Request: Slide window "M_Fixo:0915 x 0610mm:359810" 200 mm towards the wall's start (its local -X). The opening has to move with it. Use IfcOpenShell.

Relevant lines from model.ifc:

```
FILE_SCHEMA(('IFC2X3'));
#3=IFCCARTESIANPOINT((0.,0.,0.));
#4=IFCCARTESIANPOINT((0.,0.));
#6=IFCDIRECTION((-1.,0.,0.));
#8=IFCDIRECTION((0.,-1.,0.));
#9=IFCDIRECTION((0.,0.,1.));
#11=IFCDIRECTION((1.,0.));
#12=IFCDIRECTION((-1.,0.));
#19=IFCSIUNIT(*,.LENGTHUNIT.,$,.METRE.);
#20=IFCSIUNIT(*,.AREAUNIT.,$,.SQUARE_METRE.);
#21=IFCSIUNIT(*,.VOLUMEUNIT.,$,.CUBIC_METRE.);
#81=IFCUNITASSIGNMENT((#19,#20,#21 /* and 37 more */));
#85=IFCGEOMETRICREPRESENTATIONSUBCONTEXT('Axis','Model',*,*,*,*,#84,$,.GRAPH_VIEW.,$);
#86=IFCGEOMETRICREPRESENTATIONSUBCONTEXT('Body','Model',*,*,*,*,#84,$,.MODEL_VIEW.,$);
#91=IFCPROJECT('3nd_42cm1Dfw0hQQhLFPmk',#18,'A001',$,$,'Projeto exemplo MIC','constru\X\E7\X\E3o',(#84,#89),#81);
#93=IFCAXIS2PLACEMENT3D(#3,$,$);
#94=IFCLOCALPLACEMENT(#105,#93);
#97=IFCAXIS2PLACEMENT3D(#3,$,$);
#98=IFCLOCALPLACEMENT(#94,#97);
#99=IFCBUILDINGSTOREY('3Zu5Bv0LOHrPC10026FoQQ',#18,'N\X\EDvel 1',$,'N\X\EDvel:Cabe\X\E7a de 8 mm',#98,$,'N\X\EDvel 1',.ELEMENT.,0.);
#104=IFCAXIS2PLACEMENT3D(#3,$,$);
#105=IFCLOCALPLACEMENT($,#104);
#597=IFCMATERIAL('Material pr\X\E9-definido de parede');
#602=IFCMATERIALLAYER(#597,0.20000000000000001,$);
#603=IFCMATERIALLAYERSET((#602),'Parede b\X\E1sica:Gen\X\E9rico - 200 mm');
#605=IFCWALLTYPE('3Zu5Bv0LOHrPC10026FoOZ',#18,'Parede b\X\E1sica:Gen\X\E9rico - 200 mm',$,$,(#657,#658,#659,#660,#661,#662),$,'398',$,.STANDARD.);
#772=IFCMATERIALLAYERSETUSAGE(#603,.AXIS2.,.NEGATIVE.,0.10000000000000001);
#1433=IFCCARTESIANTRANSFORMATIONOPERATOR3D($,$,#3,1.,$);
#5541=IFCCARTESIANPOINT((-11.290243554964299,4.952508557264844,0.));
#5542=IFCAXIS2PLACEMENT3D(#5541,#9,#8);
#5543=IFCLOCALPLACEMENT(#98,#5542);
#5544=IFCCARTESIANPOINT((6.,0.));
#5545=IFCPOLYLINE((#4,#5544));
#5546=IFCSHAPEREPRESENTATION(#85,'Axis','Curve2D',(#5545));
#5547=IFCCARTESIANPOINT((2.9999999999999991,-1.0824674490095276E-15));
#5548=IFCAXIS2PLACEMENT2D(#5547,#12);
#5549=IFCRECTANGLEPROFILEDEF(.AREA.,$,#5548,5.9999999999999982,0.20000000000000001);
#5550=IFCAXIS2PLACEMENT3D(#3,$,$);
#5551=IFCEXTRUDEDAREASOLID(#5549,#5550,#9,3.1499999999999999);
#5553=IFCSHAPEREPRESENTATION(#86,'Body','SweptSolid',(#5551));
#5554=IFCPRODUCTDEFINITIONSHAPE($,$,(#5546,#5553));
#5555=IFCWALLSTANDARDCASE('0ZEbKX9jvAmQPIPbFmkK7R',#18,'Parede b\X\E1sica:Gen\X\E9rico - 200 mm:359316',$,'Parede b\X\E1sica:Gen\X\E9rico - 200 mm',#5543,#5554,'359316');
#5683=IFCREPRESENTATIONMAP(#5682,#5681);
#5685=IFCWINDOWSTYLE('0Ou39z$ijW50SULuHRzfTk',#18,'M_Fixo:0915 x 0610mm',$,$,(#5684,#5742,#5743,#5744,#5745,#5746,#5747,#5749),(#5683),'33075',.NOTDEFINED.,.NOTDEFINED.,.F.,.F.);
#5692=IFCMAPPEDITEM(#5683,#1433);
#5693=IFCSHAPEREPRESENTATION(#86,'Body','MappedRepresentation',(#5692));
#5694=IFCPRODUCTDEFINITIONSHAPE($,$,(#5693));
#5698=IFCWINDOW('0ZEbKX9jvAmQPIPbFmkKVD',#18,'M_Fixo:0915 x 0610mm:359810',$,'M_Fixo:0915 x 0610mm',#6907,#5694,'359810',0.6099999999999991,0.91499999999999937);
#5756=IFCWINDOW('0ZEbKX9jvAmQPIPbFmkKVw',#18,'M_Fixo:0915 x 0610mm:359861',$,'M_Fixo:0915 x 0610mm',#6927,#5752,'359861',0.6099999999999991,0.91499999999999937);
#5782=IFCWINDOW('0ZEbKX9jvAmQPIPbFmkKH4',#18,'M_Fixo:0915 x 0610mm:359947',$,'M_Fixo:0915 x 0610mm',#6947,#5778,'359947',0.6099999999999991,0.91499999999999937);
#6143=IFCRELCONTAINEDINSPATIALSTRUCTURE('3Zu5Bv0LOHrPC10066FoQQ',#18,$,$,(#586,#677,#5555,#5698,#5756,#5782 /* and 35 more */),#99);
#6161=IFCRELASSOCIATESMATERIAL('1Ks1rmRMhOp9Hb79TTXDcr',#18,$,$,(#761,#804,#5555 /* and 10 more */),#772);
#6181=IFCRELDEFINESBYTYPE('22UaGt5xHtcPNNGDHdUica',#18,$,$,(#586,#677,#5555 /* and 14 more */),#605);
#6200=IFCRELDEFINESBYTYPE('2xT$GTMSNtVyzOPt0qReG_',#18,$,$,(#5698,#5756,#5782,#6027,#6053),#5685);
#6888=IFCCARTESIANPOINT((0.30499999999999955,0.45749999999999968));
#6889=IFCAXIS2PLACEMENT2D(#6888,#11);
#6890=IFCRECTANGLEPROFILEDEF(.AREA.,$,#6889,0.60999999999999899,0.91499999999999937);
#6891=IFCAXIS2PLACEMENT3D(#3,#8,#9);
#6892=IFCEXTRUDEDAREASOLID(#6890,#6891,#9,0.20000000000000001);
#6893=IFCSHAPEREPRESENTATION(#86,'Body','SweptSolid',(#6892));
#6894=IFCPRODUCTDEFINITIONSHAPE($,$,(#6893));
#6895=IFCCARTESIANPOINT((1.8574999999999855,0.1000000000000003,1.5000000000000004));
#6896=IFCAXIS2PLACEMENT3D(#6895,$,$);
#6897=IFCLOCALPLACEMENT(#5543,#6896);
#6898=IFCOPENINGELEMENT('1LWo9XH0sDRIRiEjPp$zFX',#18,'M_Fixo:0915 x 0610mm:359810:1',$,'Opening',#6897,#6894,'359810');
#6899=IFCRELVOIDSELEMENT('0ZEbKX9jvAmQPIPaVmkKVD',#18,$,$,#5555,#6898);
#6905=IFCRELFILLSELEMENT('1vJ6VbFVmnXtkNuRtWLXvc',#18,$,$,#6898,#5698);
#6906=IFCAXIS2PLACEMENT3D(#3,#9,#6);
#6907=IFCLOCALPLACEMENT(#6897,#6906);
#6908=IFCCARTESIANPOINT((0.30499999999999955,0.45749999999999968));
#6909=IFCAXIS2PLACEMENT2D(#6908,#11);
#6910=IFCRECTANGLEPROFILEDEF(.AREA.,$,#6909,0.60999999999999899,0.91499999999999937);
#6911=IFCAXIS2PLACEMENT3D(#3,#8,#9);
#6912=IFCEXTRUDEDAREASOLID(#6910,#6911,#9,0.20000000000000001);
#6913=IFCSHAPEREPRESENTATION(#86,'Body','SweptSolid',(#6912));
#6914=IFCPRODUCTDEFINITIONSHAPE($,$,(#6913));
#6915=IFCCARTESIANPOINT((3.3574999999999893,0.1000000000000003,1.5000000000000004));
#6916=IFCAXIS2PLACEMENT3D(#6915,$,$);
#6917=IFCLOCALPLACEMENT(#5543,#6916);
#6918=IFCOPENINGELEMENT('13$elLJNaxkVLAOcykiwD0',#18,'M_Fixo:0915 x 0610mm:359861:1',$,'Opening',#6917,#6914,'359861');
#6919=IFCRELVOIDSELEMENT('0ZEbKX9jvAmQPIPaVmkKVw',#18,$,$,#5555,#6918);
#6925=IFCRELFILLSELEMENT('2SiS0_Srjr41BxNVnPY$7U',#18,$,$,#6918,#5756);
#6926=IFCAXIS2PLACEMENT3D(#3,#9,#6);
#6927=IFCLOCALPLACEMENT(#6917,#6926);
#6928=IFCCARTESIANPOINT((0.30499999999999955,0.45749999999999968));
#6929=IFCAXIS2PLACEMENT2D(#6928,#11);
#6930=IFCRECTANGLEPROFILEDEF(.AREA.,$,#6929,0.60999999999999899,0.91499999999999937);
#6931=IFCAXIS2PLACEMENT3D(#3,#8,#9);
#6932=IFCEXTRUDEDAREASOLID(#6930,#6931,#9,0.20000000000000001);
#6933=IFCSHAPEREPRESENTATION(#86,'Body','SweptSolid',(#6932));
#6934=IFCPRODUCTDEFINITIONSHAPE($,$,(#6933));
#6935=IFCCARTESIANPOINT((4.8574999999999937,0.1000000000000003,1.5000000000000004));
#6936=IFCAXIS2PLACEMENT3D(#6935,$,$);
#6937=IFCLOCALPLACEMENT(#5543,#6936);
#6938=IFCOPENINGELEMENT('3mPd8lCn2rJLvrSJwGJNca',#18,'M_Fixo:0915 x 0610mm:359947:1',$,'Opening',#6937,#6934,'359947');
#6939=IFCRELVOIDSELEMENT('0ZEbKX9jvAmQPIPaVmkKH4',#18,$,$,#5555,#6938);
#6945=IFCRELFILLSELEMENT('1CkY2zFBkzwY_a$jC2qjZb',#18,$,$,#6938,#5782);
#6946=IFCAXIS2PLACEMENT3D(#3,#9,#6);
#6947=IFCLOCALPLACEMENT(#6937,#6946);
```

```python
import ifcopenshell
import ifcopenshell.api.geometry
import ifcopenshell.util.placement

model = ifcopenshell.open("model.ifc")

window = model.by_guid("0ZEbKX9jvAmQPIPbFmkKVD")
opening = window.FillsVoids[0].RelatingOpeningElement
wall = opening.VoidsElements[0].RelatingBuildingElement

wall_matrix = ifcopenshell.util.placement.get_local_placement(wall.ObjectPlacement)
shift = wall_matrix[:3, 0] * -0.2
before = ifcopenshell.util.placement.get_local_placement(window.ObjectPlacement)[:3, 3].copy()

# The window is placed relative to its opening, so it follows when the opening moves.
matrix = ifcopenshell.util.placement.get_local_placement(opening.ObjectPlacement)
matrix[:3, 3] += shift
ifcopenshell.api.geometry.edit_object_placement(
    model, product=opening, matrix=matrix, is_si=False, should_transform_children=True
)

after = ifcopenshell.util.placement.get_local_placement(window.ObjectPlacement)[:3, 3]
print("window moved by", (after - before).round(3) + 0.0)

model.write("model-out.ifc")
```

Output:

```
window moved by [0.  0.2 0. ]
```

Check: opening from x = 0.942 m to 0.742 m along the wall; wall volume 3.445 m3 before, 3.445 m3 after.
